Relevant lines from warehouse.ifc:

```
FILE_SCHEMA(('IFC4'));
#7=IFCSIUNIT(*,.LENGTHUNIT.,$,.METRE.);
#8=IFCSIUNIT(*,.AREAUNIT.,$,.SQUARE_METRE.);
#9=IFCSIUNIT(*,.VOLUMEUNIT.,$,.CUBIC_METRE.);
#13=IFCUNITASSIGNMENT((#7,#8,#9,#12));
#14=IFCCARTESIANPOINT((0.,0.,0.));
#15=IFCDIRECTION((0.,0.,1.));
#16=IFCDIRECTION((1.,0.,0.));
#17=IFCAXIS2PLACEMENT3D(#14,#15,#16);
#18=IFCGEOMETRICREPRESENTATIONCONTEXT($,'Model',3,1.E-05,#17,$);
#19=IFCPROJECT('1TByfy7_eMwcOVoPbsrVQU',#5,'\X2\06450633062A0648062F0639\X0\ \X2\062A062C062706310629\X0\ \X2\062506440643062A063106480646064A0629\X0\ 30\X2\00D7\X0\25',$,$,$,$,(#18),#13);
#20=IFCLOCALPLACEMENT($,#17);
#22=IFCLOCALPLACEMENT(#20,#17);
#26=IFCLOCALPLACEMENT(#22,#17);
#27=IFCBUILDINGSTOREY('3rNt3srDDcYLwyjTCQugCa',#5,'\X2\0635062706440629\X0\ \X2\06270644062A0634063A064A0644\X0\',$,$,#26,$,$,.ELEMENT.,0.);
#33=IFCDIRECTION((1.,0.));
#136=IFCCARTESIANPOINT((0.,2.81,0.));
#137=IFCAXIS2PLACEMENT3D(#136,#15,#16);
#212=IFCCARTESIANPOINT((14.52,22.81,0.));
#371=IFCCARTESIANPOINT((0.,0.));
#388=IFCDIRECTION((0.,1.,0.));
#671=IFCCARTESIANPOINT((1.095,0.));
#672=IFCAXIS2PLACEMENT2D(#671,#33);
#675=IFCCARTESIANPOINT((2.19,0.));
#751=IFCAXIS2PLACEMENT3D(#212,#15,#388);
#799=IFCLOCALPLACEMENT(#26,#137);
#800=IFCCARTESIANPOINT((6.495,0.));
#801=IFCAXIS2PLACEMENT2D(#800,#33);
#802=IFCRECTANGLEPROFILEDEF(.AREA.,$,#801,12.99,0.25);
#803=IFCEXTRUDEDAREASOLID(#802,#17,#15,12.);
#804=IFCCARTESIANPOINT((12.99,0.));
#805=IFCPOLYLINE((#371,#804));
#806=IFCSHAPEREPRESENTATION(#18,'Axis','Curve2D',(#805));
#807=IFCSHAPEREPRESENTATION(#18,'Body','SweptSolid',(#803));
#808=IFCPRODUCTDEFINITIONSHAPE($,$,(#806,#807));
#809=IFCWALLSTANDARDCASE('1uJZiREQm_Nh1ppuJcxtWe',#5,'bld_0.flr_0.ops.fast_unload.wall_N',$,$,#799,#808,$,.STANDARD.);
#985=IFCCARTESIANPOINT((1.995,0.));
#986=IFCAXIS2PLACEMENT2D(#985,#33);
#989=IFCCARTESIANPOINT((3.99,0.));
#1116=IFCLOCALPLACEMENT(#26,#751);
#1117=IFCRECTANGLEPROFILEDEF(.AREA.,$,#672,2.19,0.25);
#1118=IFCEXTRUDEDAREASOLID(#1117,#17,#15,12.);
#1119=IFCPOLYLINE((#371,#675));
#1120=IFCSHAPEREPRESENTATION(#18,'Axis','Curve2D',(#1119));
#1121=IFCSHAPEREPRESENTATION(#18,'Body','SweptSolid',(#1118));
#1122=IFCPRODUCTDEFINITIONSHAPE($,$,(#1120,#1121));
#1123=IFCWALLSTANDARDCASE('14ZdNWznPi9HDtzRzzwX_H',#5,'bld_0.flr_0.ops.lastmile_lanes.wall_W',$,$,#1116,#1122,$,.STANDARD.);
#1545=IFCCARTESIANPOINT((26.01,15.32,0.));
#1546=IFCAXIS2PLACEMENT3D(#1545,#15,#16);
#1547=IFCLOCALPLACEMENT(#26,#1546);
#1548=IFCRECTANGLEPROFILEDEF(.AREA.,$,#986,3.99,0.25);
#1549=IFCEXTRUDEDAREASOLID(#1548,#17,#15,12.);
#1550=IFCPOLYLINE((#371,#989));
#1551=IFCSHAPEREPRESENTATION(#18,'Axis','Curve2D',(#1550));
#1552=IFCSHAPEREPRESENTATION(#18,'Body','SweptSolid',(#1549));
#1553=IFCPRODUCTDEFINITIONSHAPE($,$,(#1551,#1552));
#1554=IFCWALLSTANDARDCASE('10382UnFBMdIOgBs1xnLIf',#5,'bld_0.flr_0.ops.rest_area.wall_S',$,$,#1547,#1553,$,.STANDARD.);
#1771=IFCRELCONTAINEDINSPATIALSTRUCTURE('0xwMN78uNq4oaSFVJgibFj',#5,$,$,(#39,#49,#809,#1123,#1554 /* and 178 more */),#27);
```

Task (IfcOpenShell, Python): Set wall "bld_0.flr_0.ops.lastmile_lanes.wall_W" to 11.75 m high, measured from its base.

```python
import ifcopenshell
import ifcopenshell.geom
import ifcopenshell.util.shape
import ifcopenshell.util.unit

model = ifcopenshell.open("warehouse.ifc")
unit_scale = ifcopenshell.util.unit.calculate_unit_scale(model)
settings = ifcopenshell.geom.settings()


def volume(element):
    """Net volume in cubic metres, openings subtracted."""
    shape = ifcopenshell.geom.create_shape(settings, element)
    return ifcopenshell.util.shape.get_volume(shape.geometry)


wall = model.by_guid("14ZdNWznPi9HDtzRzzwX_H")
before = volume(wall)

body = next(r for r in wall.Representation.Representations if r.RepresentationIdentifier == "Body")
solid = body.Items[0]
old_height = solid.Depth
solid.Depth = 11.75 / unit_scale
after = volume(wall)

print(f"height {old_height:g} -> {solid.Depth:g}, volume {before:.3f} -> {after:.3f} m3")

model.write("warehouse_updated.ifc")
```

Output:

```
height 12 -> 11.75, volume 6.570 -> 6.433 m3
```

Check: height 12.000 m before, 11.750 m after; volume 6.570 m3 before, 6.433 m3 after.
